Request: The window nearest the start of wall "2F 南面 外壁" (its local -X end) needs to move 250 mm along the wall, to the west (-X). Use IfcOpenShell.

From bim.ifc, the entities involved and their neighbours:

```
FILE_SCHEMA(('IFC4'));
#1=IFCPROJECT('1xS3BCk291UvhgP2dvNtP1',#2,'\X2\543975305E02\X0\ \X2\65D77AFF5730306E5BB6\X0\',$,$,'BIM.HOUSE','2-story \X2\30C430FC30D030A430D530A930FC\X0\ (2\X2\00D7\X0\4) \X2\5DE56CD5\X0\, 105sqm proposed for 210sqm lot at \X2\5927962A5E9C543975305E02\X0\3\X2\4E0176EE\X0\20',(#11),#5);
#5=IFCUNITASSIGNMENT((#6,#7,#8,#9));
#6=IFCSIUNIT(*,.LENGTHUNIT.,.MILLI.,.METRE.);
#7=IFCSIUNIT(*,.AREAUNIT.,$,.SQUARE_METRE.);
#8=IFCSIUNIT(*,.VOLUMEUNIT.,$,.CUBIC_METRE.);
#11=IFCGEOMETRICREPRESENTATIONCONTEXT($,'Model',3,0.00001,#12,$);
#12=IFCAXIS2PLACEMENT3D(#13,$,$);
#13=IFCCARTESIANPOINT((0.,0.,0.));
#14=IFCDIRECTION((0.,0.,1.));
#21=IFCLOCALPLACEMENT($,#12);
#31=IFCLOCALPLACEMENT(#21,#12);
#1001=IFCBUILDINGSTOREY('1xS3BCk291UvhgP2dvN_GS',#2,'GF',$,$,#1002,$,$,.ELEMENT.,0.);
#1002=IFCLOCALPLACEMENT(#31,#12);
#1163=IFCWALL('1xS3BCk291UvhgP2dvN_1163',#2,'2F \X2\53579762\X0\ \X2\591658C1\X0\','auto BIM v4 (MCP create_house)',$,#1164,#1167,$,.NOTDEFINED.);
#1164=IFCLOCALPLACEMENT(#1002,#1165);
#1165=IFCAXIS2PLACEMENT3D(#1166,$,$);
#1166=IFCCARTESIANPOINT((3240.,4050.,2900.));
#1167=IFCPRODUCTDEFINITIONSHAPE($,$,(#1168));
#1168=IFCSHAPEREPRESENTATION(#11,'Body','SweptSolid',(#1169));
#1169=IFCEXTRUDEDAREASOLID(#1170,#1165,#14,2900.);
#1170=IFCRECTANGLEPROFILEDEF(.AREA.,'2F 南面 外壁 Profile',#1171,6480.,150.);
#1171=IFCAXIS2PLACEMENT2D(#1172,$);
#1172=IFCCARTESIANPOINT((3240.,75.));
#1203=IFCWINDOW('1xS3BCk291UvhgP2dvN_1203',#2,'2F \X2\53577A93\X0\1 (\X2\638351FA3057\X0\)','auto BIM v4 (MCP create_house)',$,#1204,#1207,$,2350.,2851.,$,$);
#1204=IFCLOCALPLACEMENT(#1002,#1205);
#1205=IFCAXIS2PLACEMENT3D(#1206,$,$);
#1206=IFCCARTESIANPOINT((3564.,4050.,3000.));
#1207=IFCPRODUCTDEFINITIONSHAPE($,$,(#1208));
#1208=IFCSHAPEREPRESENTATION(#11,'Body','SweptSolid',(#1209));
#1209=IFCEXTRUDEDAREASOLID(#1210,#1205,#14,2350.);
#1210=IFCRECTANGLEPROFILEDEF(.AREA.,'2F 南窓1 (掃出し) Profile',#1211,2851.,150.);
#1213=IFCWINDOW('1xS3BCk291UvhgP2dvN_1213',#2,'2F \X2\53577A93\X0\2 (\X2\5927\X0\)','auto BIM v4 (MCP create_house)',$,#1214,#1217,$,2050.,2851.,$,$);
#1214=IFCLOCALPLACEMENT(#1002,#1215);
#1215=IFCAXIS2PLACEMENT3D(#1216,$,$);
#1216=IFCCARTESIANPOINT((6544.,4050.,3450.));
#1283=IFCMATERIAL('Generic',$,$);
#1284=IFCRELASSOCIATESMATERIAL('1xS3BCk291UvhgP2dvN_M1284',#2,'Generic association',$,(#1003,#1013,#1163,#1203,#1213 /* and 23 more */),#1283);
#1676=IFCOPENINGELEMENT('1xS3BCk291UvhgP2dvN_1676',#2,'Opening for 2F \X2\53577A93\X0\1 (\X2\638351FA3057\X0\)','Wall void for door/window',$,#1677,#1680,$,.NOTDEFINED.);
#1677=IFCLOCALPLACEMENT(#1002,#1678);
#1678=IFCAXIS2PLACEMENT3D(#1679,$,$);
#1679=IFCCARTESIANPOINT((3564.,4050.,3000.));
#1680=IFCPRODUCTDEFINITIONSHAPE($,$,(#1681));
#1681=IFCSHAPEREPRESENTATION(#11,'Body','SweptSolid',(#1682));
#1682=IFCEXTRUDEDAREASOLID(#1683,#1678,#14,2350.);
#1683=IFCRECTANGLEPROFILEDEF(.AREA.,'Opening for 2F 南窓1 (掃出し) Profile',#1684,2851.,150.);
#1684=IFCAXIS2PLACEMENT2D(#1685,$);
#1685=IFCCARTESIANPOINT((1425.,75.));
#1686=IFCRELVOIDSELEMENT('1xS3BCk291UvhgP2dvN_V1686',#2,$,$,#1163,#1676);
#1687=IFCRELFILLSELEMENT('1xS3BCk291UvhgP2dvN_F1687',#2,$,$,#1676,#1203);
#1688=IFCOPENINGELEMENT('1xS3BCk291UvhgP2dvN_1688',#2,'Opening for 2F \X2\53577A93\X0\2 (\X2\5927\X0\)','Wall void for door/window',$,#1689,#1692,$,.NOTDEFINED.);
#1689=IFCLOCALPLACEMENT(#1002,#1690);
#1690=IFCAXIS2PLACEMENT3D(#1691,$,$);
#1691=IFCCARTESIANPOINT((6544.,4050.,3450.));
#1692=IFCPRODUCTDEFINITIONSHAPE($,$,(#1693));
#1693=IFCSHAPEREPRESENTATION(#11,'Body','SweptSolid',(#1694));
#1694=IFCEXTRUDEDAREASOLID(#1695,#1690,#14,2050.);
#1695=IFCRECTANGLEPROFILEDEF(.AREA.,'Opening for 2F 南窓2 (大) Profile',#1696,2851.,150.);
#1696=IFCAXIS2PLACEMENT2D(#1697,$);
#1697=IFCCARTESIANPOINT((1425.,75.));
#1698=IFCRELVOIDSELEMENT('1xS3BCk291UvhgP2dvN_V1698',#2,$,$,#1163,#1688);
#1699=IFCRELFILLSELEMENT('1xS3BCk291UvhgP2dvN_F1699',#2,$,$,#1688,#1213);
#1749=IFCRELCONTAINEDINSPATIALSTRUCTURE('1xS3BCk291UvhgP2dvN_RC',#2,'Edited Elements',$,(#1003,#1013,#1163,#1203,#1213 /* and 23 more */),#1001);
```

```python
import ifcopenshell
import ifcopenshell.api.geometry
import ifcopenshell.util.placement
import ifcopenshell.util.unit

model = ifcopenshell.open("bim.ifc")
unit_scale = ifcopenshell.util.unit.calculate_unit_scale(model)

window = model.by_guid("1xS3BCk291UvhgP2dvN_1203")
opening = window.FillsVoids[0].RelatingOpeningElement
wall = opening.VoidsElements[0].RelatingBuildingElement

wall_matrix = ifcopenshell.util.placement.get_local_placement(wall.ObjectPlacement)
shift = wall_matrix[:3, 0] * -0.25 / unit_scale
before = ifcopenshell.util.placement.get_local_placement(window.ObjectPlacement)[:3, 3].copy()

# The window is not placed relative to its opening, so move both.
for product in (opening, window):
    matrix = ifcopenshell.util.placement.get_local_placement(product.ObjectPlacement)
    matrix[:3, 3] += shift
    ifcopenshell.api.geometry.edit_object_placement(model, product=product, matrix=matrix, is_si=False)

after = ifcopenshell.util.placement.get_local_placement(window.ObjectPlacement)[:3, 3]
print("window moved by", (after - before).round(3) + 0.0)

model.write("bim-out.ifc")
```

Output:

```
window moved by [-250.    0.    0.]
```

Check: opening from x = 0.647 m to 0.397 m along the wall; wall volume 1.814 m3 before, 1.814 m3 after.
